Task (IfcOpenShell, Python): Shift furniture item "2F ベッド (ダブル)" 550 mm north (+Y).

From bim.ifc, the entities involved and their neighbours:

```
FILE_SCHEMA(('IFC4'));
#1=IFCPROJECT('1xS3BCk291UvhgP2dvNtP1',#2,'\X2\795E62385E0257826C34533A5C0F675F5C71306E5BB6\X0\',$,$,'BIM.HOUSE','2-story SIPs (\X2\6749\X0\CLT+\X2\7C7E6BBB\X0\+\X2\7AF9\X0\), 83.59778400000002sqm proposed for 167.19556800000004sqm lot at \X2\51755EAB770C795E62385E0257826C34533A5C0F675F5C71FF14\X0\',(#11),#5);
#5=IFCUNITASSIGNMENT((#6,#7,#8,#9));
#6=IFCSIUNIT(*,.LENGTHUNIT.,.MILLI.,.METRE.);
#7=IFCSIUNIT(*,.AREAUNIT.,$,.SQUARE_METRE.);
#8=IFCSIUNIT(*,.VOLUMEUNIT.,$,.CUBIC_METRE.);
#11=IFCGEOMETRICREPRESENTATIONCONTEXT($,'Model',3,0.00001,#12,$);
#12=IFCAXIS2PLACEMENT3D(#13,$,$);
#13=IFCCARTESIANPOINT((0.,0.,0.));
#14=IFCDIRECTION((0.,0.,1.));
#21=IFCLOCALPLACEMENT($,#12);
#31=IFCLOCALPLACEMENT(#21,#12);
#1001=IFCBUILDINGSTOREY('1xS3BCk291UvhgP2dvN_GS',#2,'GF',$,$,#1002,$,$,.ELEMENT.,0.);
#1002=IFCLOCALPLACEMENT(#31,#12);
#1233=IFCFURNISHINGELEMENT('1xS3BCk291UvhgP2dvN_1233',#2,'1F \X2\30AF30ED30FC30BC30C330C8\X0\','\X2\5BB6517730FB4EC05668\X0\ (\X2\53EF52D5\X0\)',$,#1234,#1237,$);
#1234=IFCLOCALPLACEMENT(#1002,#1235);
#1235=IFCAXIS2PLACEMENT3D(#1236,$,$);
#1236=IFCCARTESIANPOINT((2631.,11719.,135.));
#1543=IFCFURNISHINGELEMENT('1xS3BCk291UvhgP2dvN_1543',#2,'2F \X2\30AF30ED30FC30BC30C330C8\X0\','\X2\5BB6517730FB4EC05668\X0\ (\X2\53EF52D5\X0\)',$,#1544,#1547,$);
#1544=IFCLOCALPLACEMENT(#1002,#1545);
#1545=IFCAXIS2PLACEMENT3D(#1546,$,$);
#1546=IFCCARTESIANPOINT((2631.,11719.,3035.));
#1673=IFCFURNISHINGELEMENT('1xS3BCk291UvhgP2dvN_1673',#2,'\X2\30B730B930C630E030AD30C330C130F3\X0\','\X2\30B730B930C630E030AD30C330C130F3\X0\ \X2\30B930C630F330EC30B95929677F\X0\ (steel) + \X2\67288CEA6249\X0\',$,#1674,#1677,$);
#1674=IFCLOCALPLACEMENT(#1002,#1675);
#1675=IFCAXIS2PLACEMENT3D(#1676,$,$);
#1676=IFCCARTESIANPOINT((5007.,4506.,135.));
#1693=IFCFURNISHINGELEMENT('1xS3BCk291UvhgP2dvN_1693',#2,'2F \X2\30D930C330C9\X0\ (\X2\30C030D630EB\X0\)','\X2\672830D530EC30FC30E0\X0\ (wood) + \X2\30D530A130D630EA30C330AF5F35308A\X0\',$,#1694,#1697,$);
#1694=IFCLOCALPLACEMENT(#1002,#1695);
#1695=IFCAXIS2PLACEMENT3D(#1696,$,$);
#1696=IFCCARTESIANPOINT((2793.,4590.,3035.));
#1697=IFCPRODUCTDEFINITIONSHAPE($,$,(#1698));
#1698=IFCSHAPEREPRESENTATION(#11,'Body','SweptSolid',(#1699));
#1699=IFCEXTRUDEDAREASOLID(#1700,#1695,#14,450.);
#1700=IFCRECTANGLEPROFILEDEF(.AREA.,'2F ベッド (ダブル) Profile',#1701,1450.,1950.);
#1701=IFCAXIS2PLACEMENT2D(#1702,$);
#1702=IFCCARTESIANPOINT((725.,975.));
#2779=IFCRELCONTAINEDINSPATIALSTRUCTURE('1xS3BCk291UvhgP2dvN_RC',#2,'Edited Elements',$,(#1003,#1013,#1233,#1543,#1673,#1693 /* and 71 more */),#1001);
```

```python
import ifcopenshell
import ifcopenshell.api.geometry
import ifcopenshell.util.placement

model = ifcopenshell.open("bim.ifc")

item = model.by_guid("1xS3BCk291UvhgP2dvN_1693")
matrix = ifcopenshell.util.placement.get_local_placement(item.ObjectPlacement)
matrix[1, 3] += 550.0
ifcopenshell.api.geometry.edit_object_placement(model, product=item, matrix=matrix, is_si=False)

print(ifcopenshell.util.placement.get_local_placement(item.ObjectPlacement).round(3) + 0.0)

model.write("bim-out.ifc")
```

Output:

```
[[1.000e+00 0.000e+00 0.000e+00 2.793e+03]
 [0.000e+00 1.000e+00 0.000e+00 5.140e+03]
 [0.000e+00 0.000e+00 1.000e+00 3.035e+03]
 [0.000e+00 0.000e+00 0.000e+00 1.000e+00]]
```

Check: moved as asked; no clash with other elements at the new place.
